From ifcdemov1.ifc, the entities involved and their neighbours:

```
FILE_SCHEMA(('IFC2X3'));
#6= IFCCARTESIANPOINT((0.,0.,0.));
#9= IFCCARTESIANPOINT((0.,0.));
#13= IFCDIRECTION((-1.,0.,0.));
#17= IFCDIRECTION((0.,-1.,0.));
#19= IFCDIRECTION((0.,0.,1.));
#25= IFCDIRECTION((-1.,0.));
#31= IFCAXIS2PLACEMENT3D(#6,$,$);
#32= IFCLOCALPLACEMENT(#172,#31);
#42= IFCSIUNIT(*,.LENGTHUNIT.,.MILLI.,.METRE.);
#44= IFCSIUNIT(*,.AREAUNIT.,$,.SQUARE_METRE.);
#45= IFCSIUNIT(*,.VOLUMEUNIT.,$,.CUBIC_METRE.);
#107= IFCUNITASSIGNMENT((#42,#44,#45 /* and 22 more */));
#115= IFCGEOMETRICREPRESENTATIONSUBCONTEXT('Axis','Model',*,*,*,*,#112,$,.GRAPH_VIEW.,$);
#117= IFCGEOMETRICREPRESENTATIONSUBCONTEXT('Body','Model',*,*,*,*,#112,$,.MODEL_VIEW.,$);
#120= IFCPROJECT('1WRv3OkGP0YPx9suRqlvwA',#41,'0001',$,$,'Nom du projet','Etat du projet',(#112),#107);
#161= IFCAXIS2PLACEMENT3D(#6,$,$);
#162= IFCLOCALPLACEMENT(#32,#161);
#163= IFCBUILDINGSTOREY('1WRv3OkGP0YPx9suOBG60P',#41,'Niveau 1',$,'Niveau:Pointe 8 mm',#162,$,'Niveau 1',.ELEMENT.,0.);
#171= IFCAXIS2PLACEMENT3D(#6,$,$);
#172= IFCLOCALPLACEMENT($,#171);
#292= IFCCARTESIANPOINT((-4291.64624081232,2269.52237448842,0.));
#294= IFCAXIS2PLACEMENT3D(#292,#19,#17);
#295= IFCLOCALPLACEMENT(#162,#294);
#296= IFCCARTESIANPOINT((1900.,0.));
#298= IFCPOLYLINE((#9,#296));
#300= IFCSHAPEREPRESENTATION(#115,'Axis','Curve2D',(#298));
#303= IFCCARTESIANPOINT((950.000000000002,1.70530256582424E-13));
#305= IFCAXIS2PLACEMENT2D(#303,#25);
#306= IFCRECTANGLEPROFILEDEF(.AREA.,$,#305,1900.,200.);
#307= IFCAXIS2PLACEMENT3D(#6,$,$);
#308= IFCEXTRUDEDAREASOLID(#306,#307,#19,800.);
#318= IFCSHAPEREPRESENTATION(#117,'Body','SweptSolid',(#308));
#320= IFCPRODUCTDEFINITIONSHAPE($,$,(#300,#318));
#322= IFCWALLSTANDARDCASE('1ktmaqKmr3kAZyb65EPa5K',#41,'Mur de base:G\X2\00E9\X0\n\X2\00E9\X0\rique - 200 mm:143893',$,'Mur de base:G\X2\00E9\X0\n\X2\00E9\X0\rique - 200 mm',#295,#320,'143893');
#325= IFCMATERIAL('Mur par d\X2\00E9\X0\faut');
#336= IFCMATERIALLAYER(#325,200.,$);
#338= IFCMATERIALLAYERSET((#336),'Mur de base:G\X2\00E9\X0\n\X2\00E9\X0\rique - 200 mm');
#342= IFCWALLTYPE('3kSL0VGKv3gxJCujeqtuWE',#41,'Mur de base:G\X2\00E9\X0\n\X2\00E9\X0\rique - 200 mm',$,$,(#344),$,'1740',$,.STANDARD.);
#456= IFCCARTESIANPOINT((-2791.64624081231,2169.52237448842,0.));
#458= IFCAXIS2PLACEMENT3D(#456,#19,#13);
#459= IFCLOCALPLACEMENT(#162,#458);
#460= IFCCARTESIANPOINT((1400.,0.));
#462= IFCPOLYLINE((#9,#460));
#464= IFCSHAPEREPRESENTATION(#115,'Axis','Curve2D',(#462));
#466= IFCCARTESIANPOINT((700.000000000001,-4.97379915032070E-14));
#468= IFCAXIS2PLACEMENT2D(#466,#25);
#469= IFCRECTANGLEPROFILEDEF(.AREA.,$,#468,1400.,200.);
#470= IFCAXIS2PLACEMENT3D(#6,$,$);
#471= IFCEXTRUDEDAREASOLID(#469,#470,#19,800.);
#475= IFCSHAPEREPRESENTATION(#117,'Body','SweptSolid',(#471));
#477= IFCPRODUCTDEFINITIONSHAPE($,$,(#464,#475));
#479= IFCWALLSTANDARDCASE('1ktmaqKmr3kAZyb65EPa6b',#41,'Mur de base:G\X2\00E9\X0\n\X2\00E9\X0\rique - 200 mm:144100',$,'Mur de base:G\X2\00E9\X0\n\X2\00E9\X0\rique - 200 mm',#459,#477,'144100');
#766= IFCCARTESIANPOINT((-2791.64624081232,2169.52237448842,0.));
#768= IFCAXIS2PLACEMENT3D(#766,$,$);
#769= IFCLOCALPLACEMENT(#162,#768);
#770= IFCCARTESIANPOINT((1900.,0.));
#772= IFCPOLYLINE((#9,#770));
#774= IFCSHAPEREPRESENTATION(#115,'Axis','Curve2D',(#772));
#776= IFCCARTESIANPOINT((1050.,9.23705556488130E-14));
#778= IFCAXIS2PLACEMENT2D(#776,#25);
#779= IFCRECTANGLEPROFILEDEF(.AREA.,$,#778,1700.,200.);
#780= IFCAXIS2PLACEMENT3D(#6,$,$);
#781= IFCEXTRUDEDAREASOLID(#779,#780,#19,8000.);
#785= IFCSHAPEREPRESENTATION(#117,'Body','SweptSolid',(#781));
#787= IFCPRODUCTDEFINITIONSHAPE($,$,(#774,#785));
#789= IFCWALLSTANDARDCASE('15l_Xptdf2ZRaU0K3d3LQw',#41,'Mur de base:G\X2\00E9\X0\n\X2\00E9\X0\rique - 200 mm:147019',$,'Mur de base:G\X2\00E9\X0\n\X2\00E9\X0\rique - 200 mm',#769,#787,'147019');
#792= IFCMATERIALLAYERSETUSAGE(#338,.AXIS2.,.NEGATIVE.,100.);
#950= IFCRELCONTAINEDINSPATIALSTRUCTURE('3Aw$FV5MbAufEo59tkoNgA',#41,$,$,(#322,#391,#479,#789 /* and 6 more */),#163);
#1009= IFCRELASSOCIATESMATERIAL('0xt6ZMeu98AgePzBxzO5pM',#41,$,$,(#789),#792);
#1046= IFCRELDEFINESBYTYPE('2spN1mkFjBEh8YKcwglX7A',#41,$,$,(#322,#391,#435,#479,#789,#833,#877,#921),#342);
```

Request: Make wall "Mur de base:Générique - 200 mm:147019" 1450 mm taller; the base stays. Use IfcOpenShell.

```python
import ifcopenshell
import ifcopenshell.geom
import ifcopenshell.util.representation
import ifcopenshell.util.shape
import ifcopenshell.util.unit

model = ifcopenshell.open("ifcdemov1.ifc")
unit_scale = ifcopenshell.util.unit.calculate_unit_scale(model)
settings = ifcopenshell.geom.settings()


def volume(element):
    """Net volume in cubic metres, openings subtracted."""
    shape = ifcopenshell.geom.create_shape(settings, element)
    return ifcopenshell.util.shape.get_volume(shape.geometry)


wall = model.by_id(789)
before = volume(wall)

body = ifcopenshell.util.representation.get_representation(wall, "Model", "Body")
solid = body.Items[0]
old_height = solid.Depth
solid.Depth += 1.45 / unit_scale
after = volume(wall)

print(f"height {old_height:g} -> {solid.Depth:g}, volume {before:.3f} -> {after:.3f} m3")

model.write("ifcdemov1_updated.ifc")
```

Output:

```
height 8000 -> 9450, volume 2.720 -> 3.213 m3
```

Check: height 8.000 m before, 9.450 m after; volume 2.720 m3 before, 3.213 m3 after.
